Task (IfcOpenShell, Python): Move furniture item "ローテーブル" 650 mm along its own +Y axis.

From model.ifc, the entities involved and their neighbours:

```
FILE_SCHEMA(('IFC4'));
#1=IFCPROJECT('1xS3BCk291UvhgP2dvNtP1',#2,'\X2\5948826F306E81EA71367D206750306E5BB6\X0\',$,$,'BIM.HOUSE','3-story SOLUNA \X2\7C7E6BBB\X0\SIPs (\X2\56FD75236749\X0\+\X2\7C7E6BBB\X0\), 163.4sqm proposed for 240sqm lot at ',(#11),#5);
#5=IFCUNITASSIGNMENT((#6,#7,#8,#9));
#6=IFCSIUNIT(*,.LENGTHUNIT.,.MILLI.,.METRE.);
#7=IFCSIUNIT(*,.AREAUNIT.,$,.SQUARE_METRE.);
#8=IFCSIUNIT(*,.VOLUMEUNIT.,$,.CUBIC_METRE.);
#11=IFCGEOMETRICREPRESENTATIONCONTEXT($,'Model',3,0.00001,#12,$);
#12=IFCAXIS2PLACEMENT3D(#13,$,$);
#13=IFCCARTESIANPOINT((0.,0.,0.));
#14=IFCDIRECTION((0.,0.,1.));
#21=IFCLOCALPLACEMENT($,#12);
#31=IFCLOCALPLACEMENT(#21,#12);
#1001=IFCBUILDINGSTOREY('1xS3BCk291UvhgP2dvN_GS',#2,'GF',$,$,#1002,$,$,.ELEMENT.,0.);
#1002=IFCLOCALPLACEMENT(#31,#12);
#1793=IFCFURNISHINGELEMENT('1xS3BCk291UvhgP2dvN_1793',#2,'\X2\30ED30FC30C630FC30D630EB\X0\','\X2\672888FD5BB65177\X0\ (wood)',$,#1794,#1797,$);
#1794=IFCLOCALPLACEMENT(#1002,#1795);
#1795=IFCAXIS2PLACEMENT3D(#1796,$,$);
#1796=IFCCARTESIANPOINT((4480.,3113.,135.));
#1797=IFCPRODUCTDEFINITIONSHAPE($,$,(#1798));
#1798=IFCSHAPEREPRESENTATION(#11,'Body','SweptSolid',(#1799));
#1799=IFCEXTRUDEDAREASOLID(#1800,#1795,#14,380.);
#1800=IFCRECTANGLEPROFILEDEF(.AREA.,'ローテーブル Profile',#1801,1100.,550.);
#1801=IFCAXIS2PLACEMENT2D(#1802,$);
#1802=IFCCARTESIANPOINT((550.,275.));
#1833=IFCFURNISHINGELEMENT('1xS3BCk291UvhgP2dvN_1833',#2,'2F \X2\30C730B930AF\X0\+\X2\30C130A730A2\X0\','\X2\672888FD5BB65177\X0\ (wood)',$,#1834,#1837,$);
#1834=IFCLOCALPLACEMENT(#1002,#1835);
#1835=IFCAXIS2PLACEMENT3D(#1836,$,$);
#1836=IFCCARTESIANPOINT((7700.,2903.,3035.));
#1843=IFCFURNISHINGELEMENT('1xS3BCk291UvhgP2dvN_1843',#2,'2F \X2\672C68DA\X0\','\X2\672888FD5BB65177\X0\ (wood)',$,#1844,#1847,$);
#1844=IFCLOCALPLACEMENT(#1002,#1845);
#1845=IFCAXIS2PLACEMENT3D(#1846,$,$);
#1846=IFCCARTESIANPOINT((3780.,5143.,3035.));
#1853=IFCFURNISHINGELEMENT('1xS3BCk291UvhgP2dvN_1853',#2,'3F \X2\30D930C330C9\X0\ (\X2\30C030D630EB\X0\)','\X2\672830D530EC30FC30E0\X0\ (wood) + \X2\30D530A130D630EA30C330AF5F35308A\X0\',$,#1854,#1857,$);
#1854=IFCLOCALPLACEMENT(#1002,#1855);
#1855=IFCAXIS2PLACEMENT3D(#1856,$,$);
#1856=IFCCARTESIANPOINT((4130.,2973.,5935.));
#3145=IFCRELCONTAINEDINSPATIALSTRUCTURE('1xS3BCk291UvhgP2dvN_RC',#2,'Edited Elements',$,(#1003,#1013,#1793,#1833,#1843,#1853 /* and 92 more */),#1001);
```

```python
import ifcopenshell
import ifcopenshell.api.geometry
import ifcopenshell.util.placement

model = ifcopenshell.open("model.ifc")

item = model.by_id(1793)
matrix = ifcopenshell.util.placement.get_local_placement(item.ObjectPlacement)
matrix[:3, 3] += matrix[:3, 1] * 650.0
ifcopenshell.api.geometry.edit_object_placement(model, product=item, matrix=matrix, is_si=False)

print(ifcopenshell.util.placement.get_local_placement(item.ObjectPlacement).round(3) + 0.0)

model.write("model-out.ifc")
```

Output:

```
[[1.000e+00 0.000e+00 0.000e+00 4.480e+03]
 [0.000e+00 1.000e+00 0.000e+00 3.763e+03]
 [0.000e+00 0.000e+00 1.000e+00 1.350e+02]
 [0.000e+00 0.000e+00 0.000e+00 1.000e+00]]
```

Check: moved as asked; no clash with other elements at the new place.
